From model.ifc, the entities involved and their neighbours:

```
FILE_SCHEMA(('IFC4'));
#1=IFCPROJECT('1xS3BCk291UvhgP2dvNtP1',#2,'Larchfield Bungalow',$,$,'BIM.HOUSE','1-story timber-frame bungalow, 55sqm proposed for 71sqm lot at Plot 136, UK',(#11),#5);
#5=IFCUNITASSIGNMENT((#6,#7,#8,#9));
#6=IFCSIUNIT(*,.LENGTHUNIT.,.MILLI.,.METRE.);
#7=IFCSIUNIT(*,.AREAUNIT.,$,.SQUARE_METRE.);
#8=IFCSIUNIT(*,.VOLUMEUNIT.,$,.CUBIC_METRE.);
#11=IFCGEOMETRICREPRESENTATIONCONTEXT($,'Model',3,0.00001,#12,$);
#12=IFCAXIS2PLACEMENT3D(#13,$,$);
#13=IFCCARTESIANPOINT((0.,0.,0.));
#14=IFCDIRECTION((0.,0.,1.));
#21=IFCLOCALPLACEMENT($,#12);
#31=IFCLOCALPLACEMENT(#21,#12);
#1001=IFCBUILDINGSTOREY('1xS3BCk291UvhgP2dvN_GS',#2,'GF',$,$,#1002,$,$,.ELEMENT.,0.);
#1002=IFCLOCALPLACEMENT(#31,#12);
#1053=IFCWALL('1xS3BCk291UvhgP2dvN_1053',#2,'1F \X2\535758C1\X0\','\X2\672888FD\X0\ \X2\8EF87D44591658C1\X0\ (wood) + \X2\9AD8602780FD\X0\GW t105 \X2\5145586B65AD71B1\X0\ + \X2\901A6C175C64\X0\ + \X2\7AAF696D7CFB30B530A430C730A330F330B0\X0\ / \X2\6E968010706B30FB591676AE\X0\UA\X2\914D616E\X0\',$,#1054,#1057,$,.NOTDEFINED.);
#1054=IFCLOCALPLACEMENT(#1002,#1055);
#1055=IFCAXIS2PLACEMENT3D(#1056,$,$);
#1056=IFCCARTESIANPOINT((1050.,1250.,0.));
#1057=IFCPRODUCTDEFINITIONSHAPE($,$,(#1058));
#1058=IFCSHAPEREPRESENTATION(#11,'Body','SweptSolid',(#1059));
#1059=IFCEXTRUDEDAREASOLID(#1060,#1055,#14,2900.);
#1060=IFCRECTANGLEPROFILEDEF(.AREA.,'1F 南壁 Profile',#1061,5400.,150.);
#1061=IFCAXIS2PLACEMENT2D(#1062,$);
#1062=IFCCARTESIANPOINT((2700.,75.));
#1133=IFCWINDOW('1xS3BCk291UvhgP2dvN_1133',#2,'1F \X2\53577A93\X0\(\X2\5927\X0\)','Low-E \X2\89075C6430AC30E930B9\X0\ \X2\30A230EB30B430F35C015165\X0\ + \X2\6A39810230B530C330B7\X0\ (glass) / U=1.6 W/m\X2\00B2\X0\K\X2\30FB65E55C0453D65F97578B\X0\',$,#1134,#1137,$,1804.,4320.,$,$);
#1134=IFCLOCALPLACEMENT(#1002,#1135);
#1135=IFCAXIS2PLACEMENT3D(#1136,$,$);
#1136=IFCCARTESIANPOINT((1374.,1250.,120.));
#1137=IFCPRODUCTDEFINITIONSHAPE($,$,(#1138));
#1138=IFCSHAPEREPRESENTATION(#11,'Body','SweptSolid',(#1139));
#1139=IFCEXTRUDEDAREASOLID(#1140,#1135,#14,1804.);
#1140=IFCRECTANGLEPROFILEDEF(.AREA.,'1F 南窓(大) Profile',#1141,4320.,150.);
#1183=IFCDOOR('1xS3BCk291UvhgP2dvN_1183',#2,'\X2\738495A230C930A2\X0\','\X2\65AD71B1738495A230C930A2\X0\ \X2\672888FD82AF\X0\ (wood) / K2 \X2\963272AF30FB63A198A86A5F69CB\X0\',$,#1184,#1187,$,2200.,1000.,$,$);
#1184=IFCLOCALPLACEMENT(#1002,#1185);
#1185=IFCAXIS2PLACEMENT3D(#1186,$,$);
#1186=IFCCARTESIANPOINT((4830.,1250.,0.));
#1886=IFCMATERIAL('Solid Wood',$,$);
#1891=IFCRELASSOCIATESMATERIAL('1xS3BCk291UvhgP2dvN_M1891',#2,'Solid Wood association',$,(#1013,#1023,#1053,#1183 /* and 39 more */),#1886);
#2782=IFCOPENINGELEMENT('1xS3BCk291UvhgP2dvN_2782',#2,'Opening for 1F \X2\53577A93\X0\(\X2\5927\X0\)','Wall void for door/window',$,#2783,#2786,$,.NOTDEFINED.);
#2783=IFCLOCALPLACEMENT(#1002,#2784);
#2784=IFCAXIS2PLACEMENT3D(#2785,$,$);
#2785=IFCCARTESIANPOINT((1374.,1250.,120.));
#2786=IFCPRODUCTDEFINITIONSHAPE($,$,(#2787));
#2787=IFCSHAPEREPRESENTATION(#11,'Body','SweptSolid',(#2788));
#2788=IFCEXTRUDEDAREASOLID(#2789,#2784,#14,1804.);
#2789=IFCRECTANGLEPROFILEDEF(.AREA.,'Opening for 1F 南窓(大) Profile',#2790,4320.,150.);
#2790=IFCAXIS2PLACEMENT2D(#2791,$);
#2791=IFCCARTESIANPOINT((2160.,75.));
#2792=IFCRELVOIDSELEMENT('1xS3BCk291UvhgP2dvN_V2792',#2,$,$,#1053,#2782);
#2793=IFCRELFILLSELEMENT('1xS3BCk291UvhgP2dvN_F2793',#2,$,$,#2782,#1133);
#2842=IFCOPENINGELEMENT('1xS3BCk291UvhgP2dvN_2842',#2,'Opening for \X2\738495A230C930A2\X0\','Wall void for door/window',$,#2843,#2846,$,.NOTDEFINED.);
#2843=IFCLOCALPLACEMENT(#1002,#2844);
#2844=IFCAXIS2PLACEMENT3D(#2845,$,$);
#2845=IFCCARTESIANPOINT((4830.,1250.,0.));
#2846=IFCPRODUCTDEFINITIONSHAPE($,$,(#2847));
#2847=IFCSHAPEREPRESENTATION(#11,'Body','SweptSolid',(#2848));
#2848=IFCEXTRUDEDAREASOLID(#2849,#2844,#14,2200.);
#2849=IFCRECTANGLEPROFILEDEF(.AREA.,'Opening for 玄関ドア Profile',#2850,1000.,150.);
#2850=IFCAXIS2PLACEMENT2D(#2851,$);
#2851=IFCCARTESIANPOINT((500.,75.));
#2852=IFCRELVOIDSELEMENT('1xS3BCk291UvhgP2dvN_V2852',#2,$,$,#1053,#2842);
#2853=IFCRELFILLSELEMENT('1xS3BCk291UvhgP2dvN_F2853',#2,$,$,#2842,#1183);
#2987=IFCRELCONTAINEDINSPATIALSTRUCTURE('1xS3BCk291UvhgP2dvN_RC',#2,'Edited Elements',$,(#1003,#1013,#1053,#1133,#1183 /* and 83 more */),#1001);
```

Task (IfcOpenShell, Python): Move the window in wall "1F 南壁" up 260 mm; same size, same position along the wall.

```python
import numpy as np
import ifcopenshell
import ifcopenshell.api.geometry
import ifcopenshell.util.placement
import ifcopenshell.util.unit

model = ifcopenshell.open("model.ifc")
unit_scale = ifcopenshell.util.unit.calculate_unit_scale(model)

window = model.by_guid("1xS3BCk291UvhgP2dvN_1133")
opening = window.FillsVoids[0].RelatingOpeningElement
dz = 260.0

shift = np.array([0.0, 0.0, dz])
# The window is not placed relative to its opening, so move both.
for product in (opening, window):
    matrix = ifcopenshell.util.placement.get_local_placement(product.ObjectPlacement)
    matrix[:3, 3] += shift
    ifcopenshell.api.geometry.edit_object_placement(model, product=product, matrix=matrix, is_si=False)

print(f"moved by {dz * unit_scale:+.3f} m")

model.write("model_rev.ifc")
```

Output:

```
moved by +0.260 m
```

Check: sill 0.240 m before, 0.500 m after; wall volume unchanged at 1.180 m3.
